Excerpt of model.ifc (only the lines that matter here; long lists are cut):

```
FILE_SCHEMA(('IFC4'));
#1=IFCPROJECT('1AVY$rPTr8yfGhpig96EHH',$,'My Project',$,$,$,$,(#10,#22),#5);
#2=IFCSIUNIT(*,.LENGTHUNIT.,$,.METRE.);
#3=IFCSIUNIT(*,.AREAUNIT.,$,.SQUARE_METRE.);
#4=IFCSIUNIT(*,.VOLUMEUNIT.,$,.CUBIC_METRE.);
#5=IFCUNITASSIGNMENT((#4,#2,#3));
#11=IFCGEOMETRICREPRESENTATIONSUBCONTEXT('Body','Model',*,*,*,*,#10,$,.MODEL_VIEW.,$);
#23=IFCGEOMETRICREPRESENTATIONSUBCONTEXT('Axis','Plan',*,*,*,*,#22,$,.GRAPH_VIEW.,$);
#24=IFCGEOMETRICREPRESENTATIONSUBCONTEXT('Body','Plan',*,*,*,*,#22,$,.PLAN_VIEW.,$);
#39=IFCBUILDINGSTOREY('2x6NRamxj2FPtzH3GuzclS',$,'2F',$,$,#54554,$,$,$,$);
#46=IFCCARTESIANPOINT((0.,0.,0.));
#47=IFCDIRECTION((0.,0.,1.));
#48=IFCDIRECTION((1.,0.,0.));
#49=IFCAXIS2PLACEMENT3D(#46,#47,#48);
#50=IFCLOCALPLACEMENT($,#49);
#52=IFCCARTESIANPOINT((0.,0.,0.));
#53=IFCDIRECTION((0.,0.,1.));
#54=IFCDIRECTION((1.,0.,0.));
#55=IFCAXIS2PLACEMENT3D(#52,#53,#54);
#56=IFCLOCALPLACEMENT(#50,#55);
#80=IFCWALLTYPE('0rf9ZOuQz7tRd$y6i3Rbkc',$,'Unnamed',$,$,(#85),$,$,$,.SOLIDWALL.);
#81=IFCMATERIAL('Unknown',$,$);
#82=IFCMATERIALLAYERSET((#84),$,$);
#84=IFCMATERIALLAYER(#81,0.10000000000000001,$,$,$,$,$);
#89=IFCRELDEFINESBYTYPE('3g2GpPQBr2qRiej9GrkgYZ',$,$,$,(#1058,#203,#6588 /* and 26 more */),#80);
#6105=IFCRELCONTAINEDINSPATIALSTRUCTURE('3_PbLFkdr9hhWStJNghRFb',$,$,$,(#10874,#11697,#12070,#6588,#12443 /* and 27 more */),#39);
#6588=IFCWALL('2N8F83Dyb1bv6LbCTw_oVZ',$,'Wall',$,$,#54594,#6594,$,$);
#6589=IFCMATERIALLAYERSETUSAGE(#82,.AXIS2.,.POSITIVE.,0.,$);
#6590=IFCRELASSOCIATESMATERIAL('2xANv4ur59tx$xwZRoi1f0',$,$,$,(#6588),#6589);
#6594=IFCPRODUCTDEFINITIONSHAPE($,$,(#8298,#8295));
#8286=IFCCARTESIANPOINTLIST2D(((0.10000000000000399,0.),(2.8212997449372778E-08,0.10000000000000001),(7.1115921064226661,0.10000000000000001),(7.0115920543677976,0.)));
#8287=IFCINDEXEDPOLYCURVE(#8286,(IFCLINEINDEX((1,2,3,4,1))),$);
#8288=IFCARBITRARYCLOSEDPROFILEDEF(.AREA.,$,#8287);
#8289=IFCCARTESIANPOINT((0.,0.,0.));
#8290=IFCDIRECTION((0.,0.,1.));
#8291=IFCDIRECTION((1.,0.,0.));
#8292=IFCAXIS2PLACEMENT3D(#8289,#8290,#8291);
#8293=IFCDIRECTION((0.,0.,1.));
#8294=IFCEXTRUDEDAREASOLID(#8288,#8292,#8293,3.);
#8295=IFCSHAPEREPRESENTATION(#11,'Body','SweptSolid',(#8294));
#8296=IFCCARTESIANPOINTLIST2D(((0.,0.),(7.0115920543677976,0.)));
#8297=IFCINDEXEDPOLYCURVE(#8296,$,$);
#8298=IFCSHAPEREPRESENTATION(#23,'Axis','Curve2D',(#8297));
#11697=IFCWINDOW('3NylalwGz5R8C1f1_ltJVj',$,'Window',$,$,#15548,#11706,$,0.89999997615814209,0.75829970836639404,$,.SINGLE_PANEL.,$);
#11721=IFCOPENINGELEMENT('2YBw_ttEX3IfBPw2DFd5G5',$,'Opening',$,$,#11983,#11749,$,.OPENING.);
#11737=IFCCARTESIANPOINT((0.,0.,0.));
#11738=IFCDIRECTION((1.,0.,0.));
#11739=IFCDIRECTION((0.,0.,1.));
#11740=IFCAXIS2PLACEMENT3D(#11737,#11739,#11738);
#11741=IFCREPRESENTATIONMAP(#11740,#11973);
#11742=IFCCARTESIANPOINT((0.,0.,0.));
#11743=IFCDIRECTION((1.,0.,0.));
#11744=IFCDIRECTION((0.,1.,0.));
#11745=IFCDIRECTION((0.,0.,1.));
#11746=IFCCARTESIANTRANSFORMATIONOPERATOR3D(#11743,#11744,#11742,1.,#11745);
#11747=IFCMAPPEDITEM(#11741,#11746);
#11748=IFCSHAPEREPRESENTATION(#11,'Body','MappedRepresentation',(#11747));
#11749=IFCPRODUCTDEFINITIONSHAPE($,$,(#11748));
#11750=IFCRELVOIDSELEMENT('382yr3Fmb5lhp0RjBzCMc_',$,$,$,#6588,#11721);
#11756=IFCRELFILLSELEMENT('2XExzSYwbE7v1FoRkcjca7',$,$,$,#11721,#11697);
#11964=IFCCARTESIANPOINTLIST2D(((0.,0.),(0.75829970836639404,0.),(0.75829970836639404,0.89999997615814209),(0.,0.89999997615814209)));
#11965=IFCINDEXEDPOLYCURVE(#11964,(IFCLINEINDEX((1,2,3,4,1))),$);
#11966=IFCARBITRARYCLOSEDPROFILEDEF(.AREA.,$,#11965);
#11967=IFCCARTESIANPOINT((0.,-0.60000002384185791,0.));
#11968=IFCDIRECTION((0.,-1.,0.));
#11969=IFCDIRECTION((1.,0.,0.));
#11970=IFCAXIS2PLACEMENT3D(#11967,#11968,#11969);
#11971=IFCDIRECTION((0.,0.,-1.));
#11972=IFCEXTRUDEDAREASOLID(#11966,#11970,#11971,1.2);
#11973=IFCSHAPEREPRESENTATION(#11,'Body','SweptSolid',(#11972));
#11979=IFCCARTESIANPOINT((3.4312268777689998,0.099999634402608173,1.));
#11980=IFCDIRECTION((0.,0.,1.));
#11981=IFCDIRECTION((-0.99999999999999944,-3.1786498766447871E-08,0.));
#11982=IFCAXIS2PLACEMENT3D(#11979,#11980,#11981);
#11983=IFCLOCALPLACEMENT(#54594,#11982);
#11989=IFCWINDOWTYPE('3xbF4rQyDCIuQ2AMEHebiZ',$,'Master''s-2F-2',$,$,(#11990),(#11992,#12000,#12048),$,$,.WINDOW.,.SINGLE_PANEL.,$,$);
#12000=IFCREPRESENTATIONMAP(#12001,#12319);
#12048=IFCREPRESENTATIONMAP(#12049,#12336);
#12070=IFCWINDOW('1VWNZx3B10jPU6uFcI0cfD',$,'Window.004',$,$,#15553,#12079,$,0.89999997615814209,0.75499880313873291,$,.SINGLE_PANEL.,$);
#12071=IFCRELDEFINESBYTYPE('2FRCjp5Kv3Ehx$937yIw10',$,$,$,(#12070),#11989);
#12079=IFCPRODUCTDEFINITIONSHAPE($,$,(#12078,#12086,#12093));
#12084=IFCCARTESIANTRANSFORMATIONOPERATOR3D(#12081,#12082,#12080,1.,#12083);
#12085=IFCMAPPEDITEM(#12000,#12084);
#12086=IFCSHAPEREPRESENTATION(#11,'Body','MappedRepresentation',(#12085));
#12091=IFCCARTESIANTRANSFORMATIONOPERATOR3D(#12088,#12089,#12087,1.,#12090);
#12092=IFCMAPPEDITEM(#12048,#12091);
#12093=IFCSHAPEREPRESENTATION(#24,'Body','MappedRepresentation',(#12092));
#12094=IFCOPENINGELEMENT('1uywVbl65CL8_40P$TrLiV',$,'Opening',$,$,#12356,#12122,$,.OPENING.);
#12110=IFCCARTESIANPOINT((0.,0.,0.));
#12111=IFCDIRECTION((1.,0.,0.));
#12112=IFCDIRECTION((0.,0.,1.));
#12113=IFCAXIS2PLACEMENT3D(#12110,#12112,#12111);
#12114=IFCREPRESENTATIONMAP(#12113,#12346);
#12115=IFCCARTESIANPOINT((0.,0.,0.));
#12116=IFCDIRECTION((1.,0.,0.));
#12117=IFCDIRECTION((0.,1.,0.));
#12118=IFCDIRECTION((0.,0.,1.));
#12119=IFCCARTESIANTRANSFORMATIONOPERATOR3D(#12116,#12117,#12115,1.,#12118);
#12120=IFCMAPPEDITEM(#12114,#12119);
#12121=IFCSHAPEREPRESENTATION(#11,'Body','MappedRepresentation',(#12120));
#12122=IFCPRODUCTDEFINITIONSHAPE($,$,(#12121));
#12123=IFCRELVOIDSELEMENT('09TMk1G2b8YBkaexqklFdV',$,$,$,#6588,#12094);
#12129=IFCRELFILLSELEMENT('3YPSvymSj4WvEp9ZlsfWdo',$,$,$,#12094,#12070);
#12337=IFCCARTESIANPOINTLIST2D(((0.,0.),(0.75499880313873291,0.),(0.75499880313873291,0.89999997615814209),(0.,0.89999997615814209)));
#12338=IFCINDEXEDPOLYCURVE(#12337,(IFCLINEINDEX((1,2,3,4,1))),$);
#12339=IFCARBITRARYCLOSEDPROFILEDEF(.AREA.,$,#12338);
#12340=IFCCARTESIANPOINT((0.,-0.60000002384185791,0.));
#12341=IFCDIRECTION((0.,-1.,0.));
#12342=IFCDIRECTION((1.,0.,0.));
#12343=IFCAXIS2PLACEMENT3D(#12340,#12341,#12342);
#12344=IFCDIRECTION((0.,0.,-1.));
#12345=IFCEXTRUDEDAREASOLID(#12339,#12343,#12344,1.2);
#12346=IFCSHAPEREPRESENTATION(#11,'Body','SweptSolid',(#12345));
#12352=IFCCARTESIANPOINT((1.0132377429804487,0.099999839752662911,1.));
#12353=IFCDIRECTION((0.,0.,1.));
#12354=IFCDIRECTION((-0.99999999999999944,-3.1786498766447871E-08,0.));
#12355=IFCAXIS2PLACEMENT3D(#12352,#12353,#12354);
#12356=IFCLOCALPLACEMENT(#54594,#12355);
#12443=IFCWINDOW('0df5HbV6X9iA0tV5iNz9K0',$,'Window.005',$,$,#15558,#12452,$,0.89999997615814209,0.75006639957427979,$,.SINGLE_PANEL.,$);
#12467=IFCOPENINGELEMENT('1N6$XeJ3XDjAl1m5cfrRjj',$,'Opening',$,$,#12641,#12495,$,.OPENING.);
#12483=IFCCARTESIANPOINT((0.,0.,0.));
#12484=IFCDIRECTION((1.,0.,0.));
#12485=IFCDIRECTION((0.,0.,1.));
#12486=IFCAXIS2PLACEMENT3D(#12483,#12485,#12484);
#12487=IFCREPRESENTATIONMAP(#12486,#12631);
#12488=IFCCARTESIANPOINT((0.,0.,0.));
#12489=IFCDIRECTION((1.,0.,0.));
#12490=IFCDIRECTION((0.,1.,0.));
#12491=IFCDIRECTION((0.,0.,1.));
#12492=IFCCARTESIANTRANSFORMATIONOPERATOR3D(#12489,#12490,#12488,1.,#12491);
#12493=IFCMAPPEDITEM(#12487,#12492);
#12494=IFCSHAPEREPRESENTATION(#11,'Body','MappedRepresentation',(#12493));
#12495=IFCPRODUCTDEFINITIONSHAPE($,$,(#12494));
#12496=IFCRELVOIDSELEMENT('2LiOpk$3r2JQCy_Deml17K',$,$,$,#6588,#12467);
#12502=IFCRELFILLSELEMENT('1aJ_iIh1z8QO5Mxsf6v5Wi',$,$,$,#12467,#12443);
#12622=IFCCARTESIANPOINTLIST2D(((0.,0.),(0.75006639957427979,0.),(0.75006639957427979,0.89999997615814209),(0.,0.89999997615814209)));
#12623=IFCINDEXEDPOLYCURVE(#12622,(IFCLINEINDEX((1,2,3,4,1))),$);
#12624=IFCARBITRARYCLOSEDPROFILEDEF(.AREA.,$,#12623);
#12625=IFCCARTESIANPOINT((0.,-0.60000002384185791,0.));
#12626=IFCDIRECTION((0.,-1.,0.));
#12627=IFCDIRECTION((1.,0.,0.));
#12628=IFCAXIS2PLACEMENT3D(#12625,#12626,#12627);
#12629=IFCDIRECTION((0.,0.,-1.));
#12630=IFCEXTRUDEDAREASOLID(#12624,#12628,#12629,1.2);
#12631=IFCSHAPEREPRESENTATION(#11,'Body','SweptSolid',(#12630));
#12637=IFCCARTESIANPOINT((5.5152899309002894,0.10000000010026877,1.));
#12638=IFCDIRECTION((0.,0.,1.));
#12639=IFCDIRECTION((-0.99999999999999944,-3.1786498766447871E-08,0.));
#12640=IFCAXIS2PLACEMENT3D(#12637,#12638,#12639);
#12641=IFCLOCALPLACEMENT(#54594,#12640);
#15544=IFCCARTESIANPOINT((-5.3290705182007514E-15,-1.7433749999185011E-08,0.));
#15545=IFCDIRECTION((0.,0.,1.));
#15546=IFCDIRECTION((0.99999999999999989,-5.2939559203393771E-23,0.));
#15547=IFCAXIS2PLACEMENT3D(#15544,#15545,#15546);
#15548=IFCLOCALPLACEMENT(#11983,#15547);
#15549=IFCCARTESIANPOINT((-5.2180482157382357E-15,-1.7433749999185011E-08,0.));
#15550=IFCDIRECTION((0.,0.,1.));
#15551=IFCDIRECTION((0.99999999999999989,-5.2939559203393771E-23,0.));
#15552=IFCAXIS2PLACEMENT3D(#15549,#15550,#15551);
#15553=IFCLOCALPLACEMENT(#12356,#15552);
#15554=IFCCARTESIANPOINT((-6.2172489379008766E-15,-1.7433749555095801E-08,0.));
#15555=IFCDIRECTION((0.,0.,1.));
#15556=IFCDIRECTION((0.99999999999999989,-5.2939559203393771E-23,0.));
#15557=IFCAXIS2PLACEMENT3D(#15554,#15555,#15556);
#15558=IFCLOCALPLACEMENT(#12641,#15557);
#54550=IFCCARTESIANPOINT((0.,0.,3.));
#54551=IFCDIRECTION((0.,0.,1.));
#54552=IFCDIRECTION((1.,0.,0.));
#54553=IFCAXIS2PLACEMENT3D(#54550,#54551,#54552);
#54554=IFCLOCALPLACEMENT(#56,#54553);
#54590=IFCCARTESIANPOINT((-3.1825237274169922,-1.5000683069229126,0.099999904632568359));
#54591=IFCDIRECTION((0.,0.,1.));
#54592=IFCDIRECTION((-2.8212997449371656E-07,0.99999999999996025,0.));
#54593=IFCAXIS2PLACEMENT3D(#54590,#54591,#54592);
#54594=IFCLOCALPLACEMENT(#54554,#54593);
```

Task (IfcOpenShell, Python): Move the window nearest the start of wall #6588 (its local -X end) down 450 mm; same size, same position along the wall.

```python
import numpy as np
import ifcopenshell
import ifcopenshell.api.geometry
import ifcopenshell.util.placement
import ifcopenshell.util.unit

model = ifcopenshell.open("model.ifc")
unit_scale = ifcopenshell.util.unit.calculate_unit_scale(model)

window = model.by_guid("1VWNZx3B10jPU6uFcI0cfD")
opening = window.FillsVoids[0].RelatingOpeningElement
dz = -0.45 / unit_scale

shift = np.array([0.0, 0.0, dz])
# The window is placed relative to its opening, so it follows when the opening moves.
matrix = ifcopenshell.util.placement.get_local_placement(opening.ObjectPlacement)
matrix[:3, 3] += shift
ifcopenshell.api.geometry.edit_object_placement(
    model, product=opening, matrix=matrix, is_si=False, should_transform_children=True
)

print(f"moved by {dz * unit_scale:+.3f} m")

model.write("model_edited.ifc")
```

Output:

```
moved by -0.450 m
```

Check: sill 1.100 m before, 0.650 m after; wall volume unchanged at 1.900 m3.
